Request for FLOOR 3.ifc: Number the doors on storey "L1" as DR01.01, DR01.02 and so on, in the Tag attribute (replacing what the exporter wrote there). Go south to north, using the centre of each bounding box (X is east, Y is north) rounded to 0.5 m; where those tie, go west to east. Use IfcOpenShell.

First a look at what the model holds.

```python
import ifcopenshell
import ifcopenshell.util.element
import ifcopenshell.util.placement

model = ifcopenshell.open("FLOOR 3.ifc")
print(model.schema)
storey = next(s for s in model.by_type("IfcBuildingStorey") if s.Name == "L1")
doors = [e for e in ifcopenshell.util.element.get_decomposition(storey) if e.is_a("IfcDoor")]
for e in sorted(doors, key=lambda e: e.id()):
    origin = ifcopenshell.util.placement.get_local_placement(e.ObjectPlacement)[:3, 3]
    print(e.id(), e.Tag, e.Name, origin.round(2) + 0.0, sep=" | ")
```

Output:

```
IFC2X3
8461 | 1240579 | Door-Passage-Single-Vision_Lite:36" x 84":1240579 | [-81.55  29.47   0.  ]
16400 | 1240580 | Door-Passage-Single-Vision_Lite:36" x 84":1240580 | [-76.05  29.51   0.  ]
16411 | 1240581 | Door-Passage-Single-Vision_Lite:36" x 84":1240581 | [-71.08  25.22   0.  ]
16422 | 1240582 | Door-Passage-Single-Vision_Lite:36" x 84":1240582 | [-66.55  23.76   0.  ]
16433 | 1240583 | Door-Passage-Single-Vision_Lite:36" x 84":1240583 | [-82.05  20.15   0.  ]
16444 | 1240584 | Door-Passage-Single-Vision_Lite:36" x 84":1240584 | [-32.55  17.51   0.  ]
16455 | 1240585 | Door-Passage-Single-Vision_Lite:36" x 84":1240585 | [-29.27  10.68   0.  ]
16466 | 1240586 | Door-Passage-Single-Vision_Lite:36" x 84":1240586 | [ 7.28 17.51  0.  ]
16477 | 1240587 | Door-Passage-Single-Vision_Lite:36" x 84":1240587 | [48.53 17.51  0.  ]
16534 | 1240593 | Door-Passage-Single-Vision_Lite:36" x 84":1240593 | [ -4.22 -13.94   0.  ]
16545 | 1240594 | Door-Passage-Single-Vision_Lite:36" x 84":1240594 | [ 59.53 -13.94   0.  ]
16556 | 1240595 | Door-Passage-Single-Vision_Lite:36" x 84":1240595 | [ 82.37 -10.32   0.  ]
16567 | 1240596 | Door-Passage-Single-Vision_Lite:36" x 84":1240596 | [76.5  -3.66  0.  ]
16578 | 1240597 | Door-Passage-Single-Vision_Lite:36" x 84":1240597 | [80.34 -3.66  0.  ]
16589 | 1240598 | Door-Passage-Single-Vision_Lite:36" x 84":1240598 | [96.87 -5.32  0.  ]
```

```python
import ifcopenshell
import ifcopenshell.geom
import ifcopenshell.util.element
import ifcopenshell.util.shape

model = ifcopenshell.open("FLOOR 3.ifc")
settings = ifcopenshell.geom.settings()
settings.set("use-world-coords", True)


def centre(element):
    shape = ifcopenshell.geom.create_shape(settings, element)
    return ifcopenshell.util.shape.get_bbox_centroid(shape.geometry)


storey = next(s for s in model.by_type("IfcBuildingStorey") if s.Name == "L1")
doors = [e for e in ifcopenshell.util.element.get_decomposition(storey) if e.is_a("IfcDoor")]

# Insertion points can sit at a corner or the storey origin, so sort by the geometry (in metres).
centres = {e: centre(e) for e in doors}
doors.sort(key=lambda e: (round(centres[e][1] / 0.5), centres[e][0]))

for i, e in enumerate(doors, start=1):
    number = f"DR01.{i:02d}"
    e.Tag = number
    print(e.id(), number)

model.write("FLOOR 3_rev.ifc")
```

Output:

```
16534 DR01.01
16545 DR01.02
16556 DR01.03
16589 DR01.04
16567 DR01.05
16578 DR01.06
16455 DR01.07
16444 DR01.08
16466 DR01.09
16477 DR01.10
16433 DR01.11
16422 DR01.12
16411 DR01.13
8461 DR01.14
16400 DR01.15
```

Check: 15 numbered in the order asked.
